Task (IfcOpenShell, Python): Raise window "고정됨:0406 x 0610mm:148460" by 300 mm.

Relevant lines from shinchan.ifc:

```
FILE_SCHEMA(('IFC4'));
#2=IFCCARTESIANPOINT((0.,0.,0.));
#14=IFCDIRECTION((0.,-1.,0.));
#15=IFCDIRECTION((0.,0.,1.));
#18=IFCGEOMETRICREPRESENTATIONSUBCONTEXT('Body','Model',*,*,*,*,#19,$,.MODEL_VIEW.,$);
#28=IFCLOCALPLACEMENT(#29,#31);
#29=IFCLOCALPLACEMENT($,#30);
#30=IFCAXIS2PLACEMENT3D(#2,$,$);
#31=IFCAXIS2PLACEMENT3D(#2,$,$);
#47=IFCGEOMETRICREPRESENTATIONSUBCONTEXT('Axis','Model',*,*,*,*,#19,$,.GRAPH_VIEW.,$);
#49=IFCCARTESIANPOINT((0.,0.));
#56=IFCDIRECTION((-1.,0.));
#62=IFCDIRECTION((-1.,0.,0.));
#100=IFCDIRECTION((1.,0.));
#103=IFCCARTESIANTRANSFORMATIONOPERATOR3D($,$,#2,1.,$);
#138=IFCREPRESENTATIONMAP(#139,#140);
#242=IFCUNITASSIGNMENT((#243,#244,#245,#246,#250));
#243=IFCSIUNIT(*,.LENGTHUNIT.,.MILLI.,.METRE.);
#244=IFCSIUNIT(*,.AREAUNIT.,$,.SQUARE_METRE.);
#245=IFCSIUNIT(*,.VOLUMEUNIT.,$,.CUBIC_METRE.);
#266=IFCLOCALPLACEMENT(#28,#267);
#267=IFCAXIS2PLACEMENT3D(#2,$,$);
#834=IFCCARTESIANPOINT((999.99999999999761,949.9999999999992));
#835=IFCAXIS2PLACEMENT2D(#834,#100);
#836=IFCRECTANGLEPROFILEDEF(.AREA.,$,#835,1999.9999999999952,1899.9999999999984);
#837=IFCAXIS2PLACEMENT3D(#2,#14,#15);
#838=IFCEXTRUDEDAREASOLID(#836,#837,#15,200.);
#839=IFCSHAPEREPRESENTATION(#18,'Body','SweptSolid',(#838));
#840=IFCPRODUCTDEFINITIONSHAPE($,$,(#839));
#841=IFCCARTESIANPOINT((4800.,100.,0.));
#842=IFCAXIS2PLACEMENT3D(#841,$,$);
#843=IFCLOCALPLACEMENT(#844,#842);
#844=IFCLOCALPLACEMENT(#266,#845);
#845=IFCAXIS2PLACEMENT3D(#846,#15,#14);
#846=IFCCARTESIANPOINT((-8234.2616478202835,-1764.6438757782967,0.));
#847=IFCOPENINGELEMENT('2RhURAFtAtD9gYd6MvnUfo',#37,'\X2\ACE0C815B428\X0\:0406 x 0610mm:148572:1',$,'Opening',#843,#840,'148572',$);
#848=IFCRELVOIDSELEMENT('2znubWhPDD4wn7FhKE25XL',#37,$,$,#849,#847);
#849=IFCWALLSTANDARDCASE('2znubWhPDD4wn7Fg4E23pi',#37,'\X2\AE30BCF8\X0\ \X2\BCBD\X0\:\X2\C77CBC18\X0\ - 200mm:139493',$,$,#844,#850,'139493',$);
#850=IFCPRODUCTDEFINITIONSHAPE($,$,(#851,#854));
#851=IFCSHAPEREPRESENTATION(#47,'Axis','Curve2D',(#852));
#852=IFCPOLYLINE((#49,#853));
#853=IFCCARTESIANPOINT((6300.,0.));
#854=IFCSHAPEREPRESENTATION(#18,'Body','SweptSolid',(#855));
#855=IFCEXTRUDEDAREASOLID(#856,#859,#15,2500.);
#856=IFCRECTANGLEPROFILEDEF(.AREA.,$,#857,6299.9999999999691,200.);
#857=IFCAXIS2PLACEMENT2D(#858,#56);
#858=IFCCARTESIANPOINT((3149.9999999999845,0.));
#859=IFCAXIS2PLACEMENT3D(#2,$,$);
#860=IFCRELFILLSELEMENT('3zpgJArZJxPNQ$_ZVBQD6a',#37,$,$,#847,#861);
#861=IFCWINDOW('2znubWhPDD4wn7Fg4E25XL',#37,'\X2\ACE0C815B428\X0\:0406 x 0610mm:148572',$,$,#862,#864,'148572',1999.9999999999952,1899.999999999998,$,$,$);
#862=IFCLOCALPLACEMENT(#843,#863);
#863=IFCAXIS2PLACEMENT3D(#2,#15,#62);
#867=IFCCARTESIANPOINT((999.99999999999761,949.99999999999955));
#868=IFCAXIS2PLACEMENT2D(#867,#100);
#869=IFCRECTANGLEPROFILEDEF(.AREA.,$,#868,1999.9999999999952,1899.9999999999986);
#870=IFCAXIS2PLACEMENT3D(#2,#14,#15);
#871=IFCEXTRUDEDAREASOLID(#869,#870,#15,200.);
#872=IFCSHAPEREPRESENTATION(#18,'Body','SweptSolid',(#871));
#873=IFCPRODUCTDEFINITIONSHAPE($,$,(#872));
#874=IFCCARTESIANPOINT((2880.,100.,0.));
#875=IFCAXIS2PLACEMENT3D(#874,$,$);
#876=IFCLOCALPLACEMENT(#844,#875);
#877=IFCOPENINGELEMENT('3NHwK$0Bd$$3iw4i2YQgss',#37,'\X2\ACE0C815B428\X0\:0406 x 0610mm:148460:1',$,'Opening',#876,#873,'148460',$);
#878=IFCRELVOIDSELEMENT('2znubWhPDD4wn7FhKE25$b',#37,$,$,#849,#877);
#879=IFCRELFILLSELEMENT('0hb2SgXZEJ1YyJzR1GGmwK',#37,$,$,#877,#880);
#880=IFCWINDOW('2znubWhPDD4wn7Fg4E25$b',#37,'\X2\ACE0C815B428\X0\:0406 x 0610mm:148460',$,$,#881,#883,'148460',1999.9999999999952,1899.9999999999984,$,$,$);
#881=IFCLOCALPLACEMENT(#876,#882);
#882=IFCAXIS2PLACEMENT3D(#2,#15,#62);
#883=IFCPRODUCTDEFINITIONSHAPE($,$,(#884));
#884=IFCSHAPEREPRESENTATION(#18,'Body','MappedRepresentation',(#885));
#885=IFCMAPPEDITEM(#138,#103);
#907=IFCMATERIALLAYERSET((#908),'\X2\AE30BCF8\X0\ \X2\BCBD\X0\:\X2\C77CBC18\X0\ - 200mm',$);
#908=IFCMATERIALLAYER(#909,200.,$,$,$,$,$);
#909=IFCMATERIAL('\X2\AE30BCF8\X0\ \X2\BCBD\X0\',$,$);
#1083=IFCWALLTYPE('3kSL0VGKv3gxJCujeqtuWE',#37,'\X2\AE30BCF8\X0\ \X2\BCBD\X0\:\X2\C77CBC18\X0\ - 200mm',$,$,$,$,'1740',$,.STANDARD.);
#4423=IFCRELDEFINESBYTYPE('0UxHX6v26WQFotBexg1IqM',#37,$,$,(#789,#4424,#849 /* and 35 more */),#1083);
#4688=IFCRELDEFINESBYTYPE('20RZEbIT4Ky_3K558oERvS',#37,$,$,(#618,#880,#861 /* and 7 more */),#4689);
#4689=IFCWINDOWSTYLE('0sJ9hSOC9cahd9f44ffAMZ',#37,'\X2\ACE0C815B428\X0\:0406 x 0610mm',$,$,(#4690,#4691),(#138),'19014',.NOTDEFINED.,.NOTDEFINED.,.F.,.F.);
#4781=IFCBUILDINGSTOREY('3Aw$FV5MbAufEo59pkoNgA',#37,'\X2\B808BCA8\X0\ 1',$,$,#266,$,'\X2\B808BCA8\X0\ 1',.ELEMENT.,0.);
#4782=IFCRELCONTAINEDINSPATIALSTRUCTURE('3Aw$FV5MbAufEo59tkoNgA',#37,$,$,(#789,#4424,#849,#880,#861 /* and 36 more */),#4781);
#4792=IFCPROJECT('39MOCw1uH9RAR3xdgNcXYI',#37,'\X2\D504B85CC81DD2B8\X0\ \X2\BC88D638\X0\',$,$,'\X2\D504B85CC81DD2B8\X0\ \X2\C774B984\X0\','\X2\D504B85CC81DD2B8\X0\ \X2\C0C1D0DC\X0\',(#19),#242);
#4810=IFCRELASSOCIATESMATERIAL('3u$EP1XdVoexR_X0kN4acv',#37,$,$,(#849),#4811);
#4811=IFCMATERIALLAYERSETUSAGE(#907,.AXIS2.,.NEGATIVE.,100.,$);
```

```python
import numpy as np
import ifcopenshell
import ifcopenshell.api.geometry
import ifcopenshell.util.placement
import ifcopenshell.util.unit

model = ifcopenshell.open("shinchan.ifc")
unit_scale = ifcopenshell.util.unit.calculate_unit_scale(model)

window = model.by_id(880)
opening = window.FillsVoids[0].RelatingOpeningElement
dz = 0.3 / unit_scale

shift = np.array([0.0, 0.0, dz])
# The window is placed relative to its opening, so it follows when the opening moves.
matrix = ifcopenshell.util.placement.get_local_placement(opening.ObjectPlacement)
matrix[:3, 3] += shift
ifcopenshell.api.geometry.edit_object_placement(
    model, product=opening, matrix=matrix, is_si=False, should_transform_children=True
)

print(f"moved by {dz * unit_scale:+.3f} m")

model.write("shinchan_rev.ifc")
```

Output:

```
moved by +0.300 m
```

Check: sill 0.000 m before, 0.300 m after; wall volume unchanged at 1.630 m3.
